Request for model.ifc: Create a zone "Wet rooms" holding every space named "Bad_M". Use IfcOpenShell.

First a look at what the model holds.

```python
import ifcopenshell

model = ifcopenshell.open("model.ifc")
print(model.schema)
seen = {}
for space in model.by_type("IfcSpace"):
    seen[space.LongName] = seen.get(space.LongName, 0) + 1
for name, count in sorted(seen.items(), key=str):
    print(count, "x", name)
print("zones:", [z.Name for z in model.by_type("IfcZone")][:20])
```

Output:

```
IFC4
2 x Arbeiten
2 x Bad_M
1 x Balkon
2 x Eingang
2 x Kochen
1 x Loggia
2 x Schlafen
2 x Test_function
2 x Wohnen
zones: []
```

```python
import ifcopenshell
import ifcopenshell.api.group
import ifcopenshell.api.root

model = ifcopenshell.open("model.ifc")

names = {"Bad_M"}
spaces = [s for s in model.by_type("IfcSpace") if s.LongName in names]

zone = ifcopenshell.api.root.create_entity(model, ifc_class="IfcZone", name="Wet rooms")
ifcopenshell.api.group.assign_group(model, products=spaces, group=zone)
print(len(spaces), "spaces in", zone.Name)

model.write("model_rev.ifc")
```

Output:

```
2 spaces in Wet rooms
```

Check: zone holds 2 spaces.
